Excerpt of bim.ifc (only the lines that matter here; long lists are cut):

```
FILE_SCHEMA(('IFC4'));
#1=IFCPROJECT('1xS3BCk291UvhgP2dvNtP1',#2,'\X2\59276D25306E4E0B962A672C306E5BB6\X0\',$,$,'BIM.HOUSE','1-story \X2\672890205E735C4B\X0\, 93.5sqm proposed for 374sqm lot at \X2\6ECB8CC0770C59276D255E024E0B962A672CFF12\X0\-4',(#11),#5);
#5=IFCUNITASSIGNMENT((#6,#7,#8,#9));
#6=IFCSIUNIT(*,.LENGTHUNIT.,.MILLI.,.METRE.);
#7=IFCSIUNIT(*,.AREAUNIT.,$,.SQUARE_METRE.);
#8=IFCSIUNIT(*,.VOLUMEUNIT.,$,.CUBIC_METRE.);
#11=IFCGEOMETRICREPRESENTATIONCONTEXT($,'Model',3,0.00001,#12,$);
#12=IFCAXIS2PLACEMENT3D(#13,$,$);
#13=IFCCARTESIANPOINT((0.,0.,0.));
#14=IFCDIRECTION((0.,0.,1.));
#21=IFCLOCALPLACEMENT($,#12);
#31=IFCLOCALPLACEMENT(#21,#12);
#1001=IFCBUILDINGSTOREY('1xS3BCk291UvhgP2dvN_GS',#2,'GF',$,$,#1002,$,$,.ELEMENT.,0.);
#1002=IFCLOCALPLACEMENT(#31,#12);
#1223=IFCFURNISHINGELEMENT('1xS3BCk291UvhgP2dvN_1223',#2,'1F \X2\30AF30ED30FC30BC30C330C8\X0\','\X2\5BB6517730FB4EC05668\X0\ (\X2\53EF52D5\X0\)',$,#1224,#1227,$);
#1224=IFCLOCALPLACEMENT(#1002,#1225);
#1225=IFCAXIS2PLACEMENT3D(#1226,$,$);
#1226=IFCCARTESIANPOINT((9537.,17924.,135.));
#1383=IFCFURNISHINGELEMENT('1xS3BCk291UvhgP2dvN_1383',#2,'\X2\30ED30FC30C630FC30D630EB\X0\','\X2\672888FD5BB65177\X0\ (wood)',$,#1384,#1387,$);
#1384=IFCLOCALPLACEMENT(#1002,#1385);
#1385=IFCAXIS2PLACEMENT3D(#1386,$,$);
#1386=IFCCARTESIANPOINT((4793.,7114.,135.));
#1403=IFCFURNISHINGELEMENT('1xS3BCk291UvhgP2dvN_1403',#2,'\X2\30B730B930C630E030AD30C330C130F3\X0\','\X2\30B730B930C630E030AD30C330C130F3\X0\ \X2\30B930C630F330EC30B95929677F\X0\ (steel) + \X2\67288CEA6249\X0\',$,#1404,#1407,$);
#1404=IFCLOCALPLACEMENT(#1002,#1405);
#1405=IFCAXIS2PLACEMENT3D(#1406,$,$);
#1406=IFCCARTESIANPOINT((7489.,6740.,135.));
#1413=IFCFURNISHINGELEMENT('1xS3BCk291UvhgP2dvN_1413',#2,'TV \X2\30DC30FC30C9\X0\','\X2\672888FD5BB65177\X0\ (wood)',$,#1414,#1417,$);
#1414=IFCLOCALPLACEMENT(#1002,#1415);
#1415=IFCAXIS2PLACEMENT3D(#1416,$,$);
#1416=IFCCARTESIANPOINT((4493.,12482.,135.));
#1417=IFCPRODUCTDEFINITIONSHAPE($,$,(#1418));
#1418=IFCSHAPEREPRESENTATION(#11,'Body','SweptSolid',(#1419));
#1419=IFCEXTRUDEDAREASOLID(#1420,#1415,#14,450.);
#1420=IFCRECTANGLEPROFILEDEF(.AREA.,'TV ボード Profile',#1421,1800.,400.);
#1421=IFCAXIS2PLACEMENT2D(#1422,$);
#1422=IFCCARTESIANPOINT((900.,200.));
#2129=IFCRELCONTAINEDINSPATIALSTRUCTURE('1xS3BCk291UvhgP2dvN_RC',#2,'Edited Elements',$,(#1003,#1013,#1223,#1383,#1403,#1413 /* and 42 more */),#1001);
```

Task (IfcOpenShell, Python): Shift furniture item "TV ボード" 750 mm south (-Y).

```python
import ifcopenshell
import ifcopenshell.api.geometry
import ifcopenshell.util.placement

model = ifcopenshell.open("bim.ifc")

item = model.by_guid("1xS3BCk291UvhgP2dvN_1413")
matrix = ifcopenshell.util.placement.get_local_placement(item.ObjectPlacement)
matrix[1, 3] -= 750.0
ifcopenshell.api.geometry.edit_object_placement(model, product=item, matrix=matrix, is_si=False)

print(ifcopenshell.util.placement.get_local_placement(item.ObjectPlacement).round(3) + 0.0)

model.write("bim_updated.ifc")
```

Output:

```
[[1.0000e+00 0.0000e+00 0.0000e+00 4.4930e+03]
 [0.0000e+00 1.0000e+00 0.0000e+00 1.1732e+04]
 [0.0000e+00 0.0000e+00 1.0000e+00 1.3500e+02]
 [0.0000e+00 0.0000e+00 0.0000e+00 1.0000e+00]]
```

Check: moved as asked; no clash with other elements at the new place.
